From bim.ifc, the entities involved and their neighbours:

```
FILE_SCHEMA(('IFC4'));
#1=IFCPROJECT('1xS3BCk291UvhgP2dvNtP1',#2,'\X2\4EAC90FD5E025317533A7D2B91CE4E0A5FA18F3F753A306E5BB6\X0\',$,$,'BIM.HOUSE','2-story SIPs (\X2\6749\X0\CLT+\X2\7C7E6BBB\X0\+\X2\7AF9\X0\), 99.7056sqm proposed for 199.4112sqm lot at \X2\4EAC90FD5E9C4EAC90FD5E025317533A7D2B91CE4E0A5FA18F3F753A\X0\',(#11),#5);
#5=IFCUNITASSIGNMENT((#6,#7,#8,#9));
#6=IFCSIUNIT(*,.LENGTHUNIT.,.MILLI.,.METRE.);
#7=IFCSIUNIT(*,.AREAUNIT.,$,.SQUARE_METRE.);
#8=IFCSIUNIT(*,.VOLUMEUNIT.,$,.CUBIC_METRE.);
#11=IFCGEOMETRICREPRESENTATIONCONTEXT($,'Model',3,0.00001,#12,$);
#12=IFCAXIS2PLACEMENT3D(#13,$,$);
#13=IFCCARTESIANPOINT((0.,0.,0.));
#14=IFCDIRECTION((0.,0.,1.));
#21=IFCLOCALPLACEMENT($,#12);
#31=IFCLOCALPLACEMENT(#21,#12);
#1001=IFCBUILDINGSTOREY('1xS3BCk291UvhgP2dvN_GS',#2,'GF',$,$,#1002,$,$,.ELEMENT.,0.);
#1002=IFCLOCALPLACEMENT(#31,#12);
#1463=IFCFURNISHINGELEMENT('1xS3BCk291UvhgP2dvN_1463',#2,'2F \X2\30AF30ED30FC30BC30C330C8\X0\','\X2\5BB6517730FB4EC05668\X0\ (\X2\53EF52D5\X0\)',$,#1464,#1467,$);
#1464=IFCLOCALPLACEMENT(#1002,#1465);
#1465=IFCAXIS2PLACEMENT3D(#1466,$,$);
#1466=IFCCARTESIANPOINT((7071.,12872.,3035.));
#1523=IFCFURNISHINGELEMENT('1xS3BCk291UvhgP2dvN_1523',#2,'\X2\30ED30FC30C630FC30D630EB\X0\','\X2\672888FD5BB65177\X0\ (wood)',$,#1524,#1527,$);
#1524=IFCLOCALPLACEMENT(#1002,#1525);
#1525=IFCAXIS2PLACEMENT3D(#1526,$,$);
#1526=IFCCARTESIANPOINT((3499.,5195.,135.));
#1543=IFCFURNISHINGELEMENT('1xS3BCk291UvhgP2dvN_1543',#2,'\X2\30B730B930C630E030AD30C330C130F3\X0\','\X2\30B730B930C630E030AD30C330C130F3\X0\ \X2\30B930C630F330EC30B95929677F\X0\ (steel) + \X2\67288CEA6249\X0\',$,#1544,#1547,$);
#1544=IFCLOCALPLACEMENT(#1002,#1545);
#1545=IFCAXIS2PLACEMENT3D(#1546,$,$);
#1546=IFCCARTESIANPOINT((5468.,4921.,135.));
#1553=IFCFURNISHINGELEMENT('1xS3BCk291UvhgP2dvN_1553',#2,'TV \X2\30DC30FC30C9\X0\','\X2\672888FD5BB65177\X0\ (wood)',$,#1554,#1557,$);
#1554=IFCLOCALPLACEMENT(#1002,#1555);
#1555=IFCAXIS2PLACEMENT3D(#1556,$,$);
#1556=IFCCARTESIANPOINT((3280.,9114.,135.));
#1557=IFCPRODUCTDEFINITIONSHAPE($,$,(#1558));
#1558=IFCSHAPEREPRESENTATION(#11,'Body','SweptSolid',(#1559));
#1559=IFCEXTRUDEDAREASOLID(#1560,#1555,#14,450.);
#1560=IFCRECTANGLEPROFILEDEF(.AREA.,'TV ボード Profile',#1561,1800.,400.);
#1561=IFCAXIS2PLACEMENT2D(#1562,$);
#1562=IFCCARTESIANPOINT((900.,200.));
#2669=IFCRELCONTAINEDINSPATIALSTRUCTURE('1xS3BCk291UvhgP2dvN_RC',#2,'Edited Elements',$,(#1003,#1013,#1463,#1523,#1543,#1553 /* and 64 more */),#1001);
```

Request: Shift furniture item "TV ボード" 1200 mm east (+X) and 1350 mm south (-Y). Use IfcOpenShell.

```python
import ifcopenshell
import ifcopenshell.api.geometry
import ifcopenshell.util.placement

model = ifcopenshell.open("bim.ifc")

item = model.by_guid("1xS3BCk291UvhgP2dvN_1553")
matrix = ifcopenshell.util.placement.get_local_placement(item.ObjectPlacement)
matrix[0, 3] += 1200.0
matrix[1, 3] -= 1350.0
ifcopenshell.api.geometry.edit_object_placement(model, product=item, matrix=matrix, is_si=False)

print(ifcopenshell.util.placement.get_local_placement(item.ObjectPlacement).round(3) + 0.0)

model.write("bim_edited.ifc")
```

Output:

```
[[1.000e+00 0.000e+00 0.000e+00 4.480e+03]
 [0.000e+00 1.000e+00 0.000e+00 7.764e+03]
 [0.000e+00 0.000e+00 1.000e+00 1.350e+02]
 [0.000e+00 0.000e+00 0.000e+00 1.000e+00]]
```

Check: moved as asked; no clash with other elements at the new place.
